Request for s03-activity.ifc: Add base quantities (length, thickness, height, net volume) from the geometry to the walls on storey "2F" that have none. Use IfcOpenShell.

First a look at what the model holds.

```python
import ifcopenshell
import ifcopenshell.util.element
import ifcopenshell.util.unit

model = ifcopenshell.open("s03-activity.ifc")
print(model.schema)
for unit_type in ("LENGTHUNIT", "AREAUNIT", "VOLUMEUNIT"):
    print(unit_type, ifcopenshell.util.unit.calculate_unit_scale(model, unit_type))
storey = next(s for s in model.by_type("IfcBuildingStorey") if s.Name == "2F")
walls = [e for e in ifcopenshell.util.element.get_decomposition(storey) if e.is_a("IfcWall")]
for e in sorted(walls, key=lambda e: e.id()):
    print(e.id(), e.is_a(), e.Name, list(ifcopenshell.util.element.get_psets(e, qtos_only=True)), sep=" | ")
```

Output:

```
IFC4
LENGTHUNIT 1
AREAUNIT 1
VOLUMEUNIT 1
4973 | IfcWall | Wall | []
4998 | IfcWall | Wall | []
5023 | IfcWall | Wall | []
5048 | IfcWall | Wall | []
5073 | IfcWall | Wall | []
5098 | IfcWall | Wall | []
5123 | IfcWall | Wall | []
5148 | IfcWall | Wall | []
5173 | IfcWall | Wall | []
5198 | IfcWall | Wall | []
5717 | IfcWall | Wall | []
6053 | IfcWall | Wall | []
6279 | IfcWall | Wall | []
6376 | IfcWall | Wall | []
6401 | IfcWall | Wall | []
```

```python
import ifcopenshell
import ifcopenshell.api.pset
import ifcopenshell.geom
import ifcopenshell.util.element
import ifcopenshell.util.shape
import ifcopenshell.util.unit

model = ifcopenshell.open("s03-activity.ifc")
unit_scale = ifcopenshell.util.unit.calculate_unit_scale(model)
volume_scale = ifcopenshell.util.unit.calculate_unit_scale(model, "VOLUMEUNIT")
settings = ifcopenshell.geom.settings()

storey = next(s for s in model.by_type("IfcBuildingStorey") if s.Name == "2F")
walls = [e for e in ifcopenshell.util.element.get_decomposition(storey) if e.is_a("IfcWall")]

for e in sorted(walls, key=lambda e: e.id()):
    if ifcopenshell.util.element.get_psets(e, qtos_only=True, should_inherit=False):
        continue
    # Geometry comes back in metres, in the element's own axes.
    shape = ifcopenshell.geom.create_shape(settings, e)
    values = {
        "Length": ifcopenshell.util.shape.get_x(shape.geometry) / unit_scale,
        "Width": ifcopenshell.util.shape.get_y(shape.geometry) / unit_scale,
        "Height": ifcopenshell.util.shape.get_z(shape.geometry) / unit_scale,
        "NetVolume": ifcopenshell.util.shape.get_volume(shape.geometry) / volume_scale,
    }
    qto = ifcopenshell.api.pset.add_qto(model, product=e, name="Qto_WallBaseQuantities")
    ifcopenshell.api.pset.edit_qto(model, qto=qto, properties=values)
    print(e.id(), {k: round(v, 3) for k, v in values.items()})

model.write("s03-activity_updated.ifc")
```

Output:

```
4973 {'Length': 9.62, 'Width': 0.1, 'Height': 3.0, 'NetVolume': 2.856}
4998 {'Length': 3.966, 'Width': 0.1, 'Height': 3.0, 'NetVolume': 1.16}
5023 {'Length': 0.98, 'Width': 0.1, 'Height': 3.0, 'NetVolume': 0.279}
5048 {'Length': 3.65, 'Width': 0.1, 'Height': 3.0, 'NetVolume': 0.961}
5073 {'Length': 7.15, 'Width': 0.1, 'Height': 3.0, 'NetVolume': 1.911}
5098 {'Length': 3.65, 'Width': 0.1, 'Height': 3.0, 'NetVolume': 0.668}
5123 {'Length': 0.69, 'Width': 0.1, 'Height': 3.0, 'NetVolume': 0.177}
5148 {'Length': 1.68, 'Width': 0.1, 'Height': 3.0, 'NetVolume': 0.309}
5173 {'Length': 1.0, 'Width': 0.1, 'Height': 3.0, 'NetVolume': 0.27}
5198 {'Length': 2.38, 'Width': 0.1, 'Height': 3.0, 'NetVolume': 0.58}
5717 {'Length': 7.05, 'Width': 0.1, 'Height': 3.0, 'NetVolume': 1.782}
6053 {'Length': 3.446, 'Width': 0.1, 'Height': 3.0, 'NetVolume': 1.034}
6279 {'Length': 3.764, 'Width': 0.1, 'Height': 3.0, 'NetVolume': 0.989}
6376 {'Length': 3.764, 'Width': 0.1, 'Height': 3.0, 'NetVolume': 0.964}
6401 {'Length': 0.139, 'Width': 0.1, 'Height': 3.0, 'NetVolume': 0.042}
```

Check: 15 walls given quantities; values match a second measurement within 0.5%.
